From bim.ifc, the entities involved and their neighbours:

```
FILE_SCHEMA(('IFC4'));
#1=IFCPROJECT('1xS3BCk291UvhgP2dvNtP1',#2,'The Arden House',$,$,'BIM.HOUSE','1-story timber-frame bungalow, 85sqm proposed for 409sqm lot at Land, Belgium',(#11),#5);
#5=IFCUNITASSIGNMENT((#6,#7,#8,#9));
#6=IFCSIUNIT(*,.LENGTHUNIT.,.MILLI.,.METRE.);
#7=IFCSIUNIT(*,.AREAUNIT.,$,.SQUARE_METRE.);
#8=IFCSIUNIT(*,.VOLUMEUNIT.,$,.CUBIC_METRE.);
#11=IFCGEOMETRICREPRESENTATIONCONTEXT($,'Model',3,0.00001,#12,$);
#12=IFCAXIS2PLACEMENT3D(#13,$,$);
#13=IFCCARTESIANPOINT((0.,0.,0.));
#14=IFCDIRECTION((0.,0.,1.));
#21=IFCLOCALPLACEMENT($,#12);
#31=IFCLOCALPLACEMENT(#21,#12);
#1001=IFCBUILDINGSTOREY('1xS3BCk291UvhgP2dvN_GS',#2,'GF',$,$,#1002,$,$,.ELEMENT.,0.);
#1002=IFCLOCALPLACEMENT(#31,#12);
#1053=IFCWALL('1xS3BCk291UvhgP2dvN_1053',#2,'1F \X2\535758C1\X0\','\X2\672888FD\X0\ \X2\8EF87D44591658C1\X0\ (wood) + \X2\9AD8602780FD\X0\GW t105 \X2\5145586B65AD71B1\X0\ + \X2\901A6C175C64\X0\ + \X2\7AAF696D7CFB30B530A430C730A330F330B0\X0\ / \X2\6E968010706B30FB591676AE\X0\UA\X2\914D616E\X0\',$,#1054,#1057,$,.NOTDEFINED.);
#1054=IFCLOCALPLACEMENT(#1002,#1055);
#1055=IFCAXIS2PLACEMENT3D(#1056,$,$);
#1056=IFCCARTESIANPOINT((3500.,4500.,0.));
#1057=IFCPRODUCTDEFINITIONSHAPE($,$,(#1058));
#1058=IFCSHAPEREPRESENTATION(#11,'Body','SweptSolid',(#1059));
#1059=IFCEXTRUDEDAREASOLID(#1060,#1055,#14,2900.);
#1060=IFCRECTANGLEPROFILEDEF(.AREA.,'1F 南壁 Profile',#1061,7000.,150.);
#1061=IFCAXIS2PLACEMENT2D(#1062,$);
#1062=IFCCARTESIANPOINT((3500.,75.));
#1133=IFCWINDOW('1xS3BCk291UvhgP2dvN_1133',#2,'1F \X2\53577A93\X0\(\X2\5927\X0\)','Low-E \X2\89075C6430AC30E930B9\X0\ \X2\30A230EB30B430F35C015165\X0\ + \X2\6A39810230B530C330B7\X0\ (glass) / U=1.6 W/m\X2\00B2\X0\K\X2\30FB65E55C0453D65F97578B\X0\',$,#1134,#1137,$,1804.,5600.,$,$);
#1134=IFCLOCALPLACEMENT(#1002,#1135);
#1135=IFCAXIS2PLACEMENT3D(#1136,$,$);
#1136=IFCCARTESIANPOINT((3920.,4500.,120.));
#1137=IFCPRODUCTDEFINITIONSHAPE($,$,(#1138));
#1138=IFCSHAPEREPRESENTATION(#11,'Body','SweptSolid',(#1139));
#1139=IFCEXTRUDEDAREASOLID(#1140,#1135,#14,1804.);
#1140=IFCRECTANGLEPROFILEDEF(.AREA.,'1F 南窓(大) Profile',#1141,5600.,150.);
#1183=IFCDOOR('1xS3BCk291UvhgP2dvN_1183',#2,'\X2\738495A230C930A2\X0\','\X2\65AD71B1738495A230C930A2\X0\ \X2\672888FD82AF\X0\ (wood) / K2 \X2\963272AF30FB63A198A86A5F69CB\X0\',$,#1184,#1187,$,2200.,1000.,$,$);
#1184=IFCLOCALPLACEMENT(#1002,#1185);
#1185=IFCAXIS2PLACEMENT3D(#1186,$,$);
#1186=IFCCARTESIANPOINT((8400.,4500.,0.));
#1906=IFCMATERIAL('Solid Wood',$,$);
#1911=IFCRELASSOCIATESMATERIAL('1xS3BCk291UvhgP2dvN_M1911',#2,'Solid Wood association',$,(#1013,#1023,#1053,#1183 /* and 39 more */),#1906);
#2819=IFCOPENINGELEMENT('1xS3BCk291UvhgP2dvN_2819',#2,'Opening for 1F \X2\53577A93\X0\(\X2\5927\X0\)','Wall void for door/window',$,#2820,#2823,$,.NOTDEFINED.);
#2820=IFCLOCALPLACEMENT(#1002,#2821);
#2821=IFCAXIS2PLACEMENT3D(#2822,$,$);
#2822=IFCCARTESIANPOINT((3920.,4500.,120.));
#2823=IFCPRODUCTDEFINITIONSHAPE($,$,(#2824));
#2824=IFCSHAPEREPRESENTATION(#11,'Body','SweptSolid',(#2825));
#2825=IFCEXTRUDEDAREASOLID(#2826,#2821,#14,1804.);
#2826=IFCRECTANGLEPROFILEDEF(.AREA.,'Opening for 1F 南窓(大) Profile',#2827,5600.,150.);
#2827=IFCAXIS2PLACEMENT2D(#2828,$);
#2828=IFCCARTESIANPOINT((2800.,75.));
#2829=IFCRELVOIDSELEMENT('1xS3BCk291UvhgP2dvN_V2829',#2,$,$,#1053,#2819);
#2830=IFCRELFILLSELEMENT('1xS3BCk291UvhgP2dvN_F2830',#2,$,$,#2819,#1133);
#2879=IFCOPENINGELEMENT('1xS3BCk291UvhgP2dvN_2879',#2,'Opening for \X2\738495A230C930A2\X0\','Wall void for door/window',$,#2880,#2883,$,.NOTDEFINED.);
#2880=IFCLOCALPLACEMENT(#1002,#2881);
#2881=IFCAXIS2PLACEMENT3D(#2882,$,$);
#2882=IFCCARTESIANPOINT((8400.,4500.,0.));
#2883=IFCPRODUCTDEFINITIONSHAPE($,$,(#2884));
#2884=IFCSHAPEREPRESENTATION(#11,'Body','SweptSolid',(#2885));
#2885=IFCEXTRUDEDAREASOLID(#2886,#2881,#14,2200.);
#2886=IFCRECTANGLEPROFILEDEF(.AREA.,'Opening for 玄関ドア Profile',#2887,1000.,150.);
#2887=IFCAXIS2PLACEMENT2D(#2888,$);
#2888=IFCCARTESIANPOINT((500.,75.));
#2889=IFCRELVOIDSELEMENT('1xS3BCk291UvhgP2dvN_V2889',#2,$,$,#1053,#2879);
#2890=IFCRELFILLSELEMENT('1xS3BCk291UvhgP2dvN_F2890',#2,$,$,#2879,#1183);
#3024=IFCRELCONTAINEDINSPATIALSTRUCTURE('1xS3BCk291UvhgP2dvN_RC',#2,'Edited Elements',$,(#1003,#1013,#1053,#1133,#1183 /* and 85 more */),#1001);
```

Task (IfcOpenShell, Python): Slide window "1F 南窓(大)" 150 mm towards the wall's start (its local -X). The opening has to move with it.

```python
import ifcopenshell
import ifcopenshell.api.geometry
import ifcopenshell.util.placement

model = ifcopenshell.open("bim.ifc")

window = model.by_guid("1xS3BCk291UvhgP2dvN_1133")
opening = window.FillsVoids[0].RelatingOpeningElement
wall = opening.VoidsElements[0].RelatingBuildingElement

wall_matrix = ifcopenshell.util.placement.get_local_placement(wall.ObjectPlacement)
shift = wall_matrix[:3, 0] * -150.0
before = ifcopenshell.util.placement.get_local_placement(window.ObjectPlacement)[:3, 3].copy()

# The window is not placed relative to its opening, so move both.
for product in (opening, window):
    matrix = ifcopenshell.util.placement.get_local_placement(product.ObjectPlacement)
    matrix[:3, 3] += shift
    ifcopenshell.api.geometry.edit_object_placement(model, product=product, matrix=matrix, is_si=False)

after = ifcopenshell.util.placement.get_local_placement(window.ObjectPlacement)[:3, 3]
print("window moved by", (after - before).round(3) + 0.0)

model.write("bim_v2.ifc")
```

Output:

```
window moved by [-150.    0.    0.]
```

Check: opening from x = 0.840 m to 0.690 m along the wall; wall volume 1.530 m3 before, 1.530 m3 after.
